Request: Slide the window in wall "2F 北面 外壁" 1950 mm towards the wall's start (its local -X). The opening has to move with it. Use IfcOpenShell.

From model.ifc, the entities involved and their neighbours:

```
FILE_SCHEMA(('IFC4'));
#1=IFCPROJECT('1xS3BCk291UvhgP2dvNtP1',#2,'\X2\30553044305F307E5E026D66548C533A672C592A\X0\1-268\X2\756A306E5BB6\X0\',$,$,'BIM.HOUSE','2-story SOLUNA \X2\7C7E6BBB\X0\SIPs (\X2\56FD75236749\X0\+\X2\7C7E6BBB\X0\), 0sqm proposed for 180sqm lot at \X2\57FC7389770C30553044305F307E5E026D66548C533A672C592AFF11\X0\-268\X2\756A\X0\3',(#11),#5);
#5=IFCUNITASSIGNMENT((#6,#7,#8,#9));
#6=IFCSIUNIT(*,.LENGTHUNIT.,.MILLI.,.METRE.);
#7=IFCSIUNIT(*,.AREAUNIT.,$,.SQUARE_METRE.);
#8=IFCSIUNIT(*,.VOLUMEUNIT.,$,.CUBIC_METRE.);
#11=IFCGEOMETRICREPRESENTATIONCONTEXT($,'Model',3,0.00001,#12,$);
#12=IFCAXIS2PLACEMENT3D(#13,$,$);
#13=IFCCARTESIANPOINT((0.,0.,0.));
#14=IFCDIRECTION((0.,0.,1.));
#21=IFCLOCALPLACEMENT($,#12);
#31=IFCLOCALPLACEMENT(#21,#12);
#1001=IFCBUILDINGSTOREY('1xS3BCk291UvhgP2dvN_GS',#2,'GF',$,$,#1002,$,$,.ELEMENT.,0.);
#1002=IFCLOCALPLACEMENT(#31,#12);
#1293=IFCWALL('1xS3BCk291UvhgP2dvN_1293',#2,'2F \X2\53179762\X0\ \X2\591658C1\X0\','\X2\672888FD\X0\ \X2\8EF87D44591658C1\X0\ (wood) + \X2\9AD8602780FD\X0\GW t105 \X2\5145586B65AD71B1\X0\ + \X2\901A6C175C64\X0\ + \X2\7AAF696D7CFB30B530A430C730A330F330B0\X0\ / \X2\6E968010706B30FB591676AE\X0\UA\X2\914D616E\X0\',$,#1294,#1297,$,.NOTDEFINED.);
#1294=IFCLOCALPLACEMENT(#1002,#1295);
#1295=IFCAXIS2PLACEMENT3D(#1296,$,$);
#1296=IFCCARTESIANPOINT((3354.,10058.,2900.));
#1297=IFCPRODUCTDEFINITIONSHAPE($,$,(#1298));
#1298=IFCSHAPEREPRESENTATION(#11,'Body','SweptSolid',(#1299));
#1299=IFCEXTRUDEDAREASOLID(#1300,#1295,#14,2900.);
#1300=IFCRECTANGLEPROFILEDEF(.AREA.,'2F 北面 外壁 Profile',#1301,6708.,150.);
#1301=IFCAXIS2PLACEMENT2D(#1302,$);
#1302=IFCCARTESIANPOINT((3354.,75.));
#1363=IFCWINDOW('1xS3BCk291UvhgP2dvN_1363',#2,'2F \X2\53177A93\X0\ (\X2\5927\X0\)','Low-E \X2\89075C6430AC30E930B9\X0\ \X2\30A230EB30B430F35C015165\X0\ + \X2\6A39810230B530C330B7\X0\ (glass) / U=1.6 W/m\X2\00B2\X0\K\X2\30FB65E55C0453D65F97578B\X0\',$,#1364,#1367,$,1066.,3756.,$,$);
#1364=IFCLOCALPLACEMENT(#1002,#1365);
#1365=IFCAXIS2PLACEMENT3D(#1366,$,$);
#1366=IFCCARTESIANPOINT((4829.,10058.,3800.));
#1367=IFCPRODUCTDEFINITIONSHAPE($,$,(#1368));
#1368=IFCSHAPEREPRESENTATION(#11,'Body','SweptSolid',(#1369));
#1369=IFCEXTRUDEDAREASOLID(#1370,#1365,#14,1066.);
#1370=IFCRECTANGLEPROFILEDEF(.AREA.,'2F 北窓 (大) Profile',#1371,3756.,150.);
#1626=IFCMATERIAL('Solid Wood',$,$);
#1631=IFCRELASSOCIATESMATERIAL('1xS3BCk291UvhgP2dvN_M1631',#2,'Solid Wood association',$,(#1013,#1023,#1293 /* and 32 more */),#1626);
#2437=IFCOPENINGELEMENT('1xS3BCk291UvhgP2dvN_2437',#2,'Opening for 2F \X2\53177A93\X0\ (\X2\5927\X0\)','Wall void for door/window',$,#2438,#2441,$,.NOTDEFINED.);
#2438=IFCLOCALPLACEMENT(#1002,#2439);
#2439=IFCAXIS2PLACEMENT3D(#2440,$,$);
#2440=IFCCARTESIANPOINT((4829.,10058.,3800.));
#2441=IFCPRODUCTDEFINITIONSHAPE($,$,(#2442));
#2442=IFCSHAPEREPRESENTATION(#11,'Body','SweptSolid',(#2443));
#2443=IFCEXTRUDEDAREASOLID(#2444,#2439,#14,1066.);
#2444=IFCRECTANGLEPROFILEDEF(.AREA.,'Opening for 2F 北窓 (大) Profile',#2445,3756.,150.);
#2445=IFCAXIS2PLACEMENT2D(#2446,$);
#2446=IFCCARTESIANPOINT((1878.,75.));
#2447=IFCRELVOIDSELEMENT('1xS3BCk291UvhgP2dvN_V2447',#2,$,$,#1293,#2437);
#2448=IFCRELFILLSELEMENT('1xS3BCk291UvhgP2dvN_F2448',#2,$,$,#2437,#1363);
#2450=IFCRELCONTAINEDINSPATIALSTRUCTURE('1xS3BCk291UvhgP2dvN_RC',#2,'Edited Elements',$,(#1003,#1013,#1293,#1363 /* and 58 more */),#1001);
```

```python
import ifcopenshell
import ifcopenshell.api.geometry
import ifcopenshell.util.placement
import ifcopenshell.util.unit

model = ifcopenshell.open("model.ifc")
unit_scale = ifcopenshell.util.unit.calculate_unit_scale(model)

window = model.by_id(1363)
opening = window.FillsVoids[0].RelatingOpeningElement
wall = opening.VoidsElements[0].RelatingBuildingElement

wall_matrix = ifcopenshell.util.placement.get_local_placement(wall.ObjectPlacement)
shift = wall_matrix[:3, 0] * -1.95 / unit_scale
before = ifcopenshell.util.placement.get_local_placement(window.ObjectPlacement)[:3, 3].copy()

# The window is not placed relative to its opening, so move both.
for product in (opening, window):
    matrix = ifcopenshell.util.placement.get_local_placement(product.ObjectPlacement)
    matrix[:3, 3] += shift
    ifcopenshell.api.geometry.edit_object_placement(model, product=product, matrix=matrix, is_si=False)

after = ifcopenshell.util.placement.get_local_placement(window.ObjectPlacement)[:3, 3]
print("window moved by", (after - before).round(3) + 0.0)

model.write("model_v2.ifc")
```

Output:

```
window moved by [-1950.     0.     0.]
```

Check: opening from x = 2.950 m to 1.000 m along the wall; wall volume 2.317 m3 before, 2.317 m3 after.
